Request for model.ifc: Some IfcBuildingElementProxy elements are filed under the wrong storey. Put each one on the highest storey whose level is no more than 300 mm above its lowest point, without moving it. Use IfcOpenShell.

First a look at what the model holds.

```python
import ifcopenshell
import ifcopenshell.util.element
import ifcopenshell.util.placement

model = ifcopenshell.open("model.ifc")
print(model.schema)
for storey in model.by_type("IfcBuildingStorey"):
    level = ifcopenshell.util.placement.get_storey_elevation(storey)
    count = sum(e.is_a("IfcBuildingElementProxy") for e in ifcopenshell.util.element.get_contained(storey))
    print(storey.id(), storey.Name, round(level, 3), count, sep=" | ")
```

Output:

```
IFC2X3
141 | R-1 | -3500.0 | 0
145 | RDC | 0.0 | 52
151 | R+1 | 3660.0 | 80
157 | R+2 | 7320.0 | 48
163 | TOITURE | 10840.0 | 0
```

```python
import ifcopenshell
import ifcopenshell.api.spatial
import ifcopenshell.geom
import ifcopenshell.util.element
import ifcopenshell.util.placement
import ifcopenshell.util.shape
import ifcopenshell.util.unit

model = ifcopenshell.open("model.ifc")
unit_scale = ifcopenshell.util.unit.calculate_unit_scale(model)
settings = ifcopenshell.geom.settings()

levels = sorted(
    ((ifcopenshell.util.placement.get_storey_elevation(s) * unit_scale, s) for s in model.by_type("IfcBuildingStorey")),
    key=lambda pair: pair[0],
)

for e in model.by_type("IfcBuildingElementProxy"):
    current = e.ContainedInStructure[0].RelatingStructure if e.ContainedInStructure else None
    if current is None or not current.is_a("IfcBuildingStorey"):
        continue
    shape = ifcopenshell.geom.create_shape(settings, e)
    bottom = ifcopenshell.util.shape.get_shape_bottom_elevation(shape, shape.geometry)
    below = [s for level, s in levels if level <= bottom + 0.3]
    storey = below[-1] if below else levels[0][1]
    if storey != current:
        # assign_container keeps the world position.
        ifcopenshell.api.spatial.assign_container(model, products=[e], relating_structure=storey)
        print(e.id(), current.Name, "->", storey.Name)

model.write("model_edited.ifc")
```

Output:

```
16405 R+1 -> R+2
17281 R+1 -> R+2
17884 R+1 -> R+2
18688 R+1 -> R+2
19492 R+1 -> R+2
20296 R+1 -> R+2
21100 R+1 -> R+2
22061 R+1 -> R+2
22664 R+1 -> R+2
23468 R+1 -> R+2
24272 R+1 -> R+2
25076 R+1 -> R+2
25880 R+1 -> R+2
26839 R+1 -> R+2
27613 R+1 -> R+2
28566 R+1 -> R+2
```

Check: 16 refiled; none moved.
